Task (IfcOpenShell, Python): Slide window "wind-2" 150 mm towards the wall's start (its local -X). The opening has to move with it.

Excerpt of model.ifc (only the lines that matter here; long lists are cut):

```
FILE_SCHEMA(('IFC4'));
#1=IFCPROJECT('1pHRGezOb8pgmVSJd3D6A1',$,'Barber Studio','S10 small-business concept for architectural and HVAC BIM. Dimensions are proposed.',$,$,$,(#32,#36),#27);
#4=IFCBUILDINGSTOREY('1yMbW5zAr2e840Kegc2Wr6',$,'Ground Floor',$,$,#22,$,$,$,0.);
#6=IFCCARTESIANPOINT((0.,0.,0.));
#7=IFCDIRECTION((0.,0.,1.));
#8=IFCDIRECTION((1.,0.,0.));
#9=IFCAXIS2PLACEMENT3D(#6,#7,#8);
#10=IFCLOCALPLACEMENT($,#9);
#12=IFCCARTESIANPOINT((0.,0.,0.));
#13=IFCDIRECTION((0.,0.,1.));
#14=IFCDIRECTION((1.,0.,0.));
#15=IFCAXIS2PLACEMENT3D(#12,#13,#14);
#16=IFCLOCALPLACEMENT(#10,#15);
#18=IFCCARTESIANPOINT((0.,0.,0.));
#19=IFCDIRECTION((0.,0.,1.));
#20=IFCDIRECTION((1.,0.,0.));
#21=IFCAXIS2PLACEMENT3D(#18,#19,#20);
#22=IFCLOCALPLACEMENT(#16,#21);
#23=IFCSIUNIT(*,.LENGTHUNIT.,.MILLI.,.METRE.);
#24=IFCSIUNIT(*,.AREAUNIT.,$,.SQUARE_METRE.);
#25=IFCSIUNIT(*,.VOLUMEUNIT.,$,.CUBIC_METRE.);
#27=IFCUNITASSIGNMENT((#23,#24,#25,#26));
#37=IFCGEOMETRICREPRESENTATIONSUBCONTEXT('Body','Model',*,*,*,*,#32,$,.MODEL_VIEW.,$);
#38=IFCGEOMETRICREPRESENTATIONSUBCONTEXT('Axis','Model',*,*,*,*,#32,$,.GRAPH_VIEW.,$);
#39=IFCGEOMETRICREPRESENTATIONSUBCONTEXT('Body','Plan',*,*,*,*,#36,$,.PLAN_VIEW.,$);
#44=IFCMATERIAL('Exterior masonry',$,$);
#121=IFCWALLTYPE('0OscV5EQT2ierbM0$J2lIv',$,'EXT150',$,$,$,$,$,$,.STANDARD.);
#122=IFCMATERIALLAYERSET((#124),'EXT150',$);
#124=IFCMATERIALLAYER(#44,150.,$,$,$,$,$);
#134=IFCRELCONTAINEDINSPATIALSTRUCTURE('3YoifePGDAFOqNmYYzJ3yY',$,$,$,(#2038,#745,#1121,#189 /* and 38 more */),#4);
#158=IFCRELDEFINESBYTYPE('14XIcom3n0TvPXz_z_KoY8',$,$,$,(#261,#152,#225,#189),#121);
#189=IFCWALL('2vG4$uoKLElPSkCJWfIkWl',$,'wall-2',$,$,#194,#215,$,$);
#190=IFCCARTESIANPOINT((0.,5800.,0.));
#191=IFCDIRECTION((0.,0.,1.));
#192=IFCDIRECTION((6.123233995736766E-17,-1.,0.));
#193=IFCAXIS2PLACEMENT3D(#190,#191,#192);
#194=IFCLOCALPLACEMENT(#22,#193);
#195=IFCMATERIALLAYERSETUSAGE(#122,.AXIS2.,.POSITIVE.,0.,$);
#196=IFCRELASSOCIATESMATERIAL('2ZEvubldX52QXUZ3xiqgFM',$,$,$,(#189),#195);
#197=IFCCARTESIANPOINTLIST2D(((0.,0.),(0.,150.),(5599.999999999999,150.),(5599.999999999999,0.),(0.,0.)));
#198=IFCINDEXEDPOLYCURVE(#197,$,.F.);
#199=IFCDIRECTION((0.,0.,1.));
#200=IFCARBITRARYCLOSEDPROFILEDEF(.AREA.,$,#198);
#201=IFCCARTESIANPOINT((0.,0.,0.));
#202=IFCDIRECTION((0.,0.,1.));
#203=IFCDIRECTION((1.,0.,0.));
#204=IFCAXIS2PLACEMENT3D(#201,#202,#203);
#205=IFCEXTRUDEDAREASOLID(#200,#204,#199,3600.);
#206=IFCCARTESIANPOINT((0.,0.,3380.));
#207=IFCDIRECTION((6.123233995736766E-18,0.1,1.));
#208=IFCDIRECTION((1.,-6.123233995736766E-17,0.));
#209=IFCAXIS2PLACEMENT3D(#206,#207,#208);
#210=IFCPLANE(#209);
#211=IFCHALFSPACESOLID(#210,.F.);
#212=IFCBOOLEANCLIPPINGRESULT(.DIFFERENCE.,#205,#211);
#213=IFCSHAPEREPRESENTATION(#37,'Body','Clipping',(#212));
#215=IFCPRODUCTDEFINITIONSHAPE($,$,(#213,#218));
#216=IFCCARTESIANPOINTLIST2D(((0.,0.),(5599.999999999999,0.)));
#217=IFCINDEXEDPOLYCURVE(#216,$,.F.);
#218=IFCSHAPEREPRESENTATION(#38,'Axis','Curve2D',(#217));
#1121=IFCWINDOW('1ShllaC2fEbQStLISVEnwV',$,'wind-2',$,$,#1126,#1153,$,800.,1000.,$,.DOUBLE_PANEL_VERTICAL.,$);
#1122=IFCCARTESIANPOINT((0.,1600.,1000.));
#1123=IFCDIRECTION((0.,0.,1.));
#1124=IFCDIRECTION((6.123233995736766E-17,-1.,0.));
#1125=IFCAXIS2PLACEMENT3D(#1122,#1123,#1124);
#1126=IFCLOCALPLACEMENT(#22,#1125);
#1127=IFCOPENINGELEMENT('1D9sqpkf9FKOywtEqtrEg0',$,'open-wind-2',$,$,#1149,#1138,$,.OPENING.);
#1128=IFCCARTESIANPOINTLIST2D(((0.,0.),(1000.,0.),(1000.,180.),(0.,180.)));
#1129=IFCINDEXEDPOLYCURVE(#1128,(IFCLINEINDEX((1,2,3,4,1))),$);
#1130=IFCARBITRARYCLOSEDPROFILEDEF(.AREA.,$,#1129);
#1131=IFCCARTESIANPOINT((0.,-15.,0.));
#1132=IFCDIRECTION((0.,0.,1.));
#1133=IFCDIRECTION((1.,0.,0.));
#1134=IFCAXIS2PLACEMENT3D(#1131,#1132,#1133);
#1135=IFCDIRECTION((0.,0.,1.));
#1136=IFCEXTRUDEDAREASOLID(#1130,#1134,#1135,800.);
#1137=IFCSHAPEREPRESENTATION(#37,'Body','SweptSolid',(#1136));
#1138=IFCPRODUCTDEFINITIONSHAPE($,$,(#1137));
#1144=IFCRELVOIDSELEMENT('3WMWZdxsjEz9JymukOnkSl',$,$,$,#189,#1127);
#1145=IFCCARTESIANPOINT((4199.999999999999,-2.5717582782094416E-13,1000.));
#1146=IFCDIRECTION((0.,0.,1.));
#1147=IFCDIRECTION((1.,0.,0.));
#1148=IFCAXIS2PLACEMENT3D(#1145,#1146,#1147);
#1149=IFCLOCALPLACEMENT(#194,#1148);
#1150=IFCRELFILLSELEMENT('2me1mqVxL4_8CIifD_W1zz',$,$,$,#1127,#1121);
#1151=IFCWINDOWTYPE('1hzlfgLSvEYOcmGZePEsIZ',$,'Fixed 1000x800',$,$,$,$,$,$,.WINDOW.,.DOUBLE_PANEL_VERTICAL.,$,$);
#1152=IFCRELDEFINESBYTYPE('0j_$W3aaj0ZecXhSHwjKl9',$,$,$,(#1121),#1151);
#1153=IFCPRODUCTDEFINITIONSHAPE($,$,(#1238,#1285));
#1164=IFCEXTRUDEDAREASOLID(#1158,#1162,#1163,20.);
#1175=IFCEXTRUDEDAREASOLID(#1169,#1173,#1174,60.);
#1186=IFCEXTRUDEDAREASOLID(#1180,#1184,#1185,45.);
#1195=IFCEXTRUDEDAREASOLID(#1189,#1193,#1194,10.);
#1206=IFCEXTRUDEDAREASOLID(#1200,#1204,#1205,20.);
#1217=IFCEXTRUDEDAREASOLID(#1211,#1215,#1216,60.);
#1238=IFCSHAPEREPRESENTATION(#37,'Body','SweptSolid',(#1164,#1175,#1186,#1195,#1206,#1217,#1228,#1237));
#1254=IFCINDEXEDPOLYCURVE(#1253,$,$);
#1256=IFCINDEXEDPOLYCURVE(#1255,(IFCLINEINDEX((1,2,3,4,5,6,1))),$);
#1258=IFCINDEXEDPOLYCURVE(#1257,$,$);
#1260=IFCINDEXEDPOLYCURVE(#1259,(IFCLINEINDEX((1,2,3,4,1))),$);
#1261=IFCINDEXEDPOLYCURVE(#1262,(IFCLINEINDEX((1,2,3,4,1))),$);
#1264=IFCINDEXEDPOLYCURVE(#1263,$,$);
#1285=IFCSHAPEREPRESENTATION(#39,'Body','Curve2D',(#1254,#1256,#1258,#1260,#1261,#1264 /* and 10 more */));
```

```python
import ifcopenshell
import ifcopenshell.api.geometry
import ifcopenshell.util.placement

model = ifcopenshell.open("model.ifc")

window = model.by_guid("1ShllaC2fEbQStLISVEnwV")
opening = window.FillsVoids[0].RelatingOpeningElement
wall = opening.VoidsElements[0].RelatingBuildingElement

wall_matrix = ifcopenshell.util.placement.get_local_placement(wall.ObjectPlacement)
shift = wall_matrix[:3, 0] * -150.0
before = ifcopenshell.util.placement.get_local_placement(window.ObjectPlacement)[:3, 3].copy()

# The window is not placed relative to its opening, so move both.
for product in (opening, window):
    matrix = ifcopenshell.util.placement.get_local_placement(product.ObjectPlacement)
    matrix[:3, 3] += shift
    ifcopenshell.api.geometry.edit_object_placement(model, product=product, matrix=matrix, is_si=False)

after = ifcopenshell.util.placement.get_local_placement(window.ObjectPlacement)[:3, 3]
print("window moved by", (after - before).round(3) + 0.0)

model.write("model_edited.ifc")
```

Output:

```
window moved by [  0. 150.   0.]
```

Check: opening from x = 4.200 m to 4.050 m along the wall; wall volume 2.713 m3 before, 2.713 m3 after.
